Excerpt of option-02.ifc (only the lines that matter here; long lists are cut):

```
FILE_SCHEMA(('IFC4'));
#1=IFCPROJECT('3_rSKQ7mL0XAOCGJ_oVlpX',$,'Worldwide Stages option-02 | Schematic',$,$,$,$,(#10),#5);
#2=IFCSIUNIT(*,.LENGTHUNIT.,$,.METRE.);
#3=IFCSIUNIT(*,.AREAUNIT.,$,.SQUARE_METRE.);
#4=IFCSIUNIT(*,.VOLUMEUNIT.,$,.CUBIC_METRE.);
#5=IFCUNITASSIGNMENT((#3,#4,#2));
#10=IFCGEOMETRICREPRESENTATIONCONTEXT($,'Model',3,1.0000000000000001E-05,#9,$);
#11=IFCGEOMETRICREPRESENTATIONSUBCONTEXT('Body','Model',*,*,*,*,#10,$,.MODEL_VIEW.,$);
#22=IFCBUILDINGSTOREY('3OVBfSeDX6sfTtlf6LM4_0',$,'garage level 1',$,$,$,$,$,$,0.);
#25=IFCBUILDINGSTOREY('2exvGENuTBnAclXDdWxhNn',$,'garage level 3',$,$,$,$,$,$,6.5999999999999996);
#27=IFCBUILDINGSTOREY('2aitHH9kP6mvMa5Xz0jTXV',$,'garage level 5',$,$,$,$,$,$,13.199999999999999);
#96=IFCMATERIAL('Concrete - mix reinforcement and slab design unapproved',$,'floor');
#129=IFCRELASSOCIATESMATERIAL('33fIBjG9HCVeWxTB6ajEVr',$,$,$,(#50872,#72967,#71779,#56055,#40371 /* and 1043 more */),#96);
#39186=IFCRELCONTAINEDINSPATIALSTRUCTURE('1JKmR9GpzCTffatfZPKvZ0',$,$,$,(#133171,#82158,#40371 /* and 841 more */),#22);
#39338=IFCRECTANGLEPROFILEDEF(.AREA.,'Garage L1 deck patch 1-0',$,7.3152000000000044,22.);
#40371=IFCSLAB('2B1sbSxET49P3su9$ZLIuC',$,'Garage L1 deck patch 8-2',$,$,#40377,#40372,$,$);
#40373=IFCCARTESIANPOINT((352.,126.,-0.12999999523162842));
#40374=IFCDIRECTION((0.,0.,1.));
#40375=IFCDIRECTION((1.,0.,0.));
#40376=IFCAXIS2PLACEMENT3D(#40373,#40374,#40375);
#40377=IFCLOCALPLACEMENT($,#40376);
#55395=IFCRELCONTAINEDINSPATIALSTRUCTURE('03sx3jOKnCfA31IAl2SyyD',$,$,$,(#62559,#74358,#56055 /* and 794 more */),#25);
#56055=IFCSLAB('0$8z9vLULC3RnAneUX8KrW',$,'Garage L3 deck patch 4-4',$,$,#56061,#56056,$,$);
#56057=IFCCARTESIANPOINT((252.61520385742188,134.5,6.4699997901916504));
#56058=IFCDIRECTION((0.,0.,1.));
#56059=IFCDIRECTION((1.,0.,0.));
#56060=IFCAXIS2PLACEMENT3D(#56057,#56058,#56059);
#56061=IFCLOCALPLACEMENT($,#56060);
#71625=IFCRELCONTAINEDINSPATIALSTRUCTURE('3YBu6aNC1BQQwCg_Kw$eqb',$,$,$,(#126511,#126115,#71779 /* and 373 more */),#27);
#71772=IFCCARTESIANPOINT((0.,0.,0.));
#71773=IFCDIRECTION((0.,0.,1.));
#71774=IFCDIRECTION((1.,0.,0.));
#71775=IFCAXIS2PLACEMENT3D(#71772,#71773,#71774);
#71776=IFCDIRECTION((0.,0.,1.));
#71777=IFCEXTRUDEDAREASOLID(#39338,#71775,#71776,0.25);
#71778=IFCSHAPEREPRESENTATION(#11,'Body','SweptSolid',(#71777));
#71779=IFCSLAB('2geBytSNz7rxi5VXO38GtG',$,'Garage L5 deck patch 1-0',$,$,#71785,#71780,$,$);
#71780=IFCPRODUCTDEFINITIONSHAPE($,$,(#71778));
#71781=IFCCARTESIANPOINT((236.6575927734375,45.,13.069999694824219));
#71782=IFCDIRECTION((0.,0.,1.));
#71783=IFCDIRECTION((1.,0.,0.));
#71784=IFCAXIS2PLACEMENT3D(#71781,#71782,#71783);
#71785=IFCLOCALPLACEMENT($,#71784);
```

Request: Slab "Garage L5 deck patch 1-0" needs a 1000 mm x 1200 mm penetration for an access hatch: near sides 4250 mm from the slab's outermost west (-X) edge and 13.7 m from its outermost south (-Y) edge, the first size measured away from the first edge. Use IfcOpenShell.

```python
import numpy as np
import ifcopenshell
import ifcopenshell.api.feature
import ifcopenshell.api.geometry
import ifcopenshell.api.root
import ifcopenshell.geom
import ifcopenshell.util.placement
import ifcopenshell.util.representation
import ifcopenshell.util.shape
import ifcopenshell.util.unit

model = ifcopenshell.open("option-02.ifc")
unit_scale = ifcopenshell.util.unit.calculate_unit_scale(model)
settings = ifcopenshell.geom.settings()


def volume(element):
    """Net volume in cubic metres, openings subtracted."""
    shape = ifcopenshell.geom.create_shape(settings, element)
    return ifcopenshell.util.shape.get_volume(shape.geometry)


slab = model.by_guid("2geBytSNz7rxi5VXO38GtG")
before = volume(slab)

# Extent in the slab's own axes, in metres. The edges named are its -X and -Y sides.
slab_shape = ifcopenshell.geom.create_shape(settings, slab)
vertices = ifcopenshell.util.shape.get_vertices(slab_shape.geometry)
x_min, y_min, bottom = vertices.min(axis=0)
top = vertices[:, 2].max()

opening = ifcopenshell.api.root.create_entity(model, ifc_class="IfcOpeningElement", name="Access hatch opening", predefined_type="OPENING")
context = ifcopenshell.util.representation.get_context(model, "Model", "Body", "MODEL_VIEW")
width, depth = 1, 1.2
outline = [(0.0, 0.0), (width, 0.0), (width, depth), (0.0, depth), (0.0, 0.0)]
# Overshoot both faces by 50 mm so the cut is clean.
shape = ifcopenshell.api.geometry.add_slab_representation(
    model, context=context, depth=top - bottom + 0.1, polyline=outline
)
ifcopenshell.api.geometry.assign_representation(model, product=opening, representation=shape)

matrix = ifcopenshell.util.placement.get_local_placement(slab.ObjectPlacement)
matrix[:, 3] = matrix @ np.append(np.array([x_min + 4.25, y_min + 13.7, bottom - 0.05]) / unit_scale, 1.0)
ifcopenshell.api.geometry.edit_object_placement(model, product=opening, matrix=matrix, is_si=False)
ifcopenshell.api.feature.add_feature(model, feature=opening, element=slab)

after = volume(slab)

print(f"slab volume {before:.3f} -> {after:.3f} m3")

model.write("option-02-out.ifc")
```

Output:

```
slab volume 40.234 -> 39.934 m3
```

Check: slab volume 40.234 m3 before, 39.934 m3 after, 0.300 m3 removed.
